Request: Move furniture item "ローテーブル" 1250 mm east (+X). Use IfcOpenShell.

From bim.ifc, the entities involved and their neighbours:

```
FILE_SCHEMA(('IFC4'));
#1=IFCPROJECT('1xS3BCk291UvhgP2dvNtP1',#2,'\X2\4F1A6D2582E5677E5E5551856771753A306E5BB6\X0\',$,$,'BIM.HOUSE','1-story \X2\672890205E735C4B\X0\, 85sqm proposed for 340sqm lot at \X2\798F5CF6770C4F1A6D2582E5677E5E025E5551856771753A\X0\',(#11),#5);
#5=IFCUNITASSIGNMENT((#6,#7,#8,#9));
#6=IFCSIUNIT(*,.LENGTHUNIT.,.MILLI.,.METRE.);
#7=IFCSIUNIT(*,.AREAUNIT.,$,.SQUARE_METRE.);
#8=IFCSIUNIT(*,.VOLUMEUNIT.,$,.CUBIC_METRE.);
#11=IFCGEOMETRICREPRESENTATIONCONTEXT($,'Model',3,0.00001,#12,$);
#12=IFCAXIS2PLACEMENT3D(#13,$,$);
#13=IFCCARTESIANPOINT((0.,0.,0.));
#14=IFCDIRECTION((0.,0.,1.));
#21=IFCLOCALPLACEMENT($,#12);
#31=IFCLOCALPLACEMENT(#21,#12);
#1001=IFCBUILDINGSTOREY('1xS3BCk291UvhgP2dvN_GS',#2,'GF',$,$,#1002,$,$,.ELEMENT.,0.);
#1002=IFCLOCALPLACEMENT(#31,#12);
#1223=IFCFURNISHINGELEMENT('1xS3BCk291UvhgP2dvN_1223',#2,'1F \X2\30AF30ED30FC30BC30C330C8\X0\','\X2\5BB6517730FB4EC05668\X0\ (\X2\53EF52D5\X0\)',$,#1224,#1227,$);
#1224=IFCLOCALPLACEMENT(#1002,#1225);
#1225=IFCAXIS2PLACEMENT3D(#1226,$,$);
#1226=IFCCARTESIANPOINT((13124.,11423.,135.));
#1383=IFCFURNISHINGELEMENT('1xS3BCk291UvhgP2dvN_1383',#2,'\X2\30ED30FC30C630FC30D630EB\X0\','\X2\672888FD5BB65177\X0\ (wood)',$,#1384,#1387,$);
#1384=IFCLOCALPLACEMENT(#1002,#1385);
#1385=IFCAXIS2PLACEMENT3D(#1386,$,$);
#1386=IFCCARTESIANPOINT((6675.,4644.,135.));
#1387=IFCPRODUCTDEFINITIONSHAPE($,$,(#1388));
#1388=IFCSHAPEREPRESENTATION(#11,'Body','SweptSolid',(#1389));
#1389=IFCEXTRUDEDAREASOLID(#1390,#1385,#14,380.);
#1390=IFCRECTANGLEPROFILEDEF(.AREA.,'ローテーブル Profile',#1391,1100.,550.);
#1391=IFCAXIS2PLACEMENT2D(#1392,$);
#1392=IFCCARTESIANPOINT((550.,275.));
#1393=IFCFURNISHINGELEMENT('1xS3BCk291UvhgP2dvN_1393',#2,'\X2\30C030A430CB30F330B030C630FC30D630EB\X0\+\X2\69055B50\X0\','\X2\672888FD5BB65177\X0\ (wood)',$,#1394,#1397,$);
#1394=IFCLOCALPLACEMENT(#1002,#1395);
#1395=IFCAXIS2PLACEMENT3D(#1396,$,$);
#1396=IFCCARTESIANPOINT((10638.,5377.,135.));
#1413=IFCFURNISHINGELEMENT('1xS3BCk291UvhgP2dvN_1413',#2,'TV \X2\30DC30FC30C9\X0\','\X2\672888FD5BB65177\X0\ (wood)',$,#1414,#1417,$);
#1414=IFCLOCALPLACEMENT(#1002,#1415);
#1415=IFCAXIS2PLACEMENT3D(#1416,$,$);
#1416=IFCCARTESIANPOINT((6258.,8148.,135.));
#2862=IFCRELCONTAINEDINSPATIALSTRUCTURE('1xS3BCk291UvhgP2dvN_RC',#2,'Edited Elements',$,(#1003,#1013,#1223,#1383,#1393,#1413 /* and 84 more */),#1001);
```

```python
import ifcopenshell
import ifcopenshell.api.geometry
import ifcopenshell.util.placement

model = ifcopenshell.open("bim.ifc")

item = model.by_guid("1xS3BCk291UvhgP2dvN_1383")
matrix = ifcopenshell.util.placement.get_local_placement(item.ObjectPlacement)
matrix[0, 3] += 1250.0
ifcopenshell.api.geometry.edit_object_placement(model, product=item, matrix=matrix, is_si=False)

print(ifcopenshell.util.placement.get_local_placement(item.ObjectPlacement).round(3) + 0.0)

model.write("bim_rev.ifc")
```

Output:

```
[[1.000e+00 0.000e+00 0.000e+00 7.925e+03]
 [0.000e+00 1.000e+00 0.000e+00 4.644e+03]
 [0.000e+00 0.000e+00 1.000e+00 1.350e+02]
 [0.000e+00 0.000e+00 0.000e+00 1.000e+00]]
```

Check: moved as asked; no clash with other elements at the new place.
